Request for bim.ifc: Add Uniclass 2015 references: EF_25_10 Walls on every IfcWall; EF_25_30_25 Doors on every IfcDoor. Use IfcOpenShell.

First a look at what the model holds.

```python
import ifcopenshell

model = ifcopenshell.open("bim.ifc")
print(model.schema)
print("classifications:", [c.Name for c in model.by_type("IfcClassification")])
for ifc_class in ("IfcDoor", "IfcRoof", "IfcStair", "IfcWall", "IfcWindow"):
    print(ifc_class, len(model.by_type(ifc_class)))
```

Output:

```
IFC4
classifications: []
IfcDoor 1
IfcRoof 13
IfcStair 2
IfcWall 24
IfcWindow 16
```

```python
import ifcopenshell
import ifcopenshell.api.classification

model = ifcopenshell.open("bim.ifc")

system = ifcopenshell.api.classification.add_classification(model, classification="Uniclass 2015")

codes = {
    "IfcWall": ("EF_25_10", "Walls"),
    "IfcDoor": ("EF_25_30_25", "Doors"),
}
for ifc_class, (code, name) in codes.items():
    products = model.by_type(ifc_class)
    ifcopenshell.api.classification.add_reference(
        model, products=products, classification=system, identification=code, name=name
    )
    print(code, len(products))

model.write("bim_updated.ifc")
```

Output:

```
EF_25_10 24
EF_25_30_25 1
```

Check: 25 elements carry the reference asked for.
